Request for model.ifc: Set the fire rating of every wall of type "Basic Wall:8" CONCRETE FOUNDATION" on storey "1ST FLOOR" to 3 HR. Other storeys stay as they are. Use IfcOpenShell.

First a look at what the model holds.

```python
import ifcopenshell
import ifcopenshell.util.element

model = ifcopenshell.open("model.ifc")
print(model.schema)
storey = next(s for s in model.by_type("IfcBuildingStorey") if s.Name == "1ST FLOOR")
walls = [e for e in ifcopenshell.util.element.get_decomposition(storey) if e.is_a("IfcWall")]
seen = {}
for e in walls:
    element_type = ifcopenshell.util.element.get_type(e)
    key = (element_type.Name if element_type != e and element_type else None, ifcopenshell.util.element.get_pset(e, "Pset_WallCommon", "FireRating"))
    seen[key] = seen.get(key, 0) + 1
for (name, value), count in sorted(seen.items(), key=str):
    print(count, "x", name, "|", value)
```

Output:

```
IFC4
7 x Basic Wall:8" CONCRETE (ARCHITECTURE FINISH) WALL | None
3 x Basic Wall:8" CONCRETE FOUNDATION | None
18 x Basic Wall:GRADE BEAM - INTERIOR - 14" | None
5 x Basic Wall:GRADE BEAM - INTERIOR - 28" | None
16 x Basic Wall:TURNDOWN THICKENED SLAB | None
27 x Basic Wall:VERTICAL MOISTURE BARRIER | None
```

```python
import ifcopenshell
import ifcopenshell.api.pset
import ifcopenshell.util.element

model = ifcopenshell.open("model.ifc")

storey = next(s for s in model.by_type("IfcBuildingStorey") if s.Name == "1ST FLOOR")
walls = [e for e in ifcopenshell.util.element.get_decomposition(storey) if e.is_a("IfcWall")]

count = 0
for e in walls:
    element_type = ifcopenshell.util.element.get_type(e)
    if element_type in (None, e) or element_type.Name != 'Basic Wall:8" CONCRETE FOUNDATION':
        continue
    # add_pset returns the element's existing set when there is one.
    pset = ifcopenshell.api.pset.add_pset(model, product=e, name="Pset_WallCommon")
    ifcopenshell.api.pset.edit_pset(model, pset=pset, properties={"FireRating": "3 HR"})
    count += 1

print(count, "walls updated")

model.write("model-out.ifc")
```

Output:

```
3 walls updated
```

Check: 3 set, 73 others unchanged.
